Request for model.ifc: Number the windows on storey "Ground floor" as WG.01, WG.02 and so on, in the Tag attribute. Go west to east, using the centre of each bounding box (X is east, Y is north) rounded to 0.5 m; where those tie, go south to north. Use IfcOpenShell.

First a look at what the model holds.

```python
import ifcopenshell
import ifcopenshell.util.element
import ifcopenshell.util.placement

model = ifcopenshell.open("model.ifc")
print(model.schema)
storey = next(s for s in model.by_type("IfcBuildingStorey") if s.Name == "Ground floor")
windows = [e for e in ifcopenshell.util.element.get_decomposition(storey) if e.is_a("IfcWindow")]
for e in sorted(windows, key=lambda e: e.id()):
    origin = ifcopenshell.util.placement.get_local_placement(e.ObjectPlacement)[:3, 3]
    print(e.id(), e.Tag, e.Name, origin.round(2) + 0.0, sep=" | ")
```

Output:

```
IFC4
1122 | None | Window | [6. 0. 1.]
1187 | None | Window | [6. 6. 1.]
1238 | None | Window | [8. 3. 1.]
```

```python
import ifcopenshell
import ifcopenshell.geom
import ifcopenshell.util.element
import ifcopenshell.util.shape

model = ifcopenshell.open("model.ifc")
settings = ifcopenshell.geom.settings()
settings.set("use-world-coords", True)


def centre(element):
    shape = ifcopenshell.geom.create_shape(settings, element)
    return ifcopenshell.util.shape.get_bbox_centroid(shape.geometry)


storey = next(s for s in model.by_type("IfcBuildingStorey") if s.Name == "Ground floor")
windows = [e for e in ifcopenshell.util.element.get_decomposition(storey) if e.is_a("IfcWindow")]

# Insertion points can sit at a corner or the storey origin, so sort by the geometry (in metres).
centres = {e: centre(e) for e in windows}
windows.sort(key=lambda e: (round(centres[e][0] / 0.5), centres[e][1]))

for i, e in enumerate(windows, start=1):
    number = f"WG.{i:02d}"
    e.Tag = number
    print(e.id(), number)

model.write("model_edited.ifc")
```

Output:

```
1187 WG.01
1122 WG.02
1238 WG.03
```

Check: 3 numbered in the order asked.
